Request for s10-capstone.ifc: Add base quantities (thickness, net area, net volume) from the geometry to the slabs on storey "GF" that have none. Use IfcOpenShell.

First a look at what the model holds.

```python
import ifcopenshell
import ifcopenshell.util.element
import ifcopenshell.util.unit

model = ifcopenshell.open("s10-capstone.ifc")
print(model.schema)
for unit_type in ("LENGTHUNIT", "AREAUNIT", "VOLUMEUNIT"):
    print(unit_type, ifcopenshell.util.unit.calculate_unit_scale(model, unit_type))
storey = next(s for s in model.by_type("IfcBuildingStorey") if s.Name == "GF")
slabs = [e for e in ifcopenshell.util.element.get_decomposition(storey) if e.is_a("IfcSlab")]
for e in sorted(slabs, key=lambda e: e.id()):
    print(e.id(), e.is_a(), e.Name, list(ifcopenshell.util.element.get_psets(e, qtos_only=True)), sep=" | ")
```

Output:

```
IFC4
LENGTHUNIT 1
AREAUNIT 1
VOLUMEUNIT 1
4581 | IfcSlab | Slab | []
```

```python
import ifcopenshell
import ifcopenshell.api.pset
import ifcopenshell.geom
import ifcopenshell.util.element
import ifcopenshell.util.shape
import ifcopenshell.util.unit

model = ifcopenshell.open("s10-capstone.ifc")
unit_scale = ifcopenshell.util.unit.calculate_unit_scale(model)
area_scale = ifcopenshell.util.unit.calculate_unit_scale(model, "AREAUNIT")
volume_scale = ifcopenshell.util.unit.calculate_unit_scale(model, "VOLUMEUNIT")
settings = ifcopenshell.geom.settings()

storey = next(s for s in model.by_type("IfcBuildingStorey") if s.Name == "GF")
slabs = [e for e in ifcopenshell.util.element.get_decomposition(storey) if e.is_a("IfcSlab")]

for e in sorted(slabs, key=lambda e: e.id()):
    if ifcopenshell.util.element.get_psets(e, qtos_only=True, should_inherit=False):
        continue
    # Geometry comes back in metres, in the element's own axes.
    shape = ifcopenshell.geom.create_shape(settings, e)
    values = {
        "Width": ifcopenshell.util.shape.get_z(shape.geometry) / unit_scale,
        "NetArea": ifcopenshell.util.shape.get_footprint_area(shape.geometry) / area_scale,
        "NetVolume": ifcopenshell.util.shape.get_volume(shape.geometry) / volume_scale,
    }
    qto = ifcopenshell.api.pset.add_qto(model, product=e, name="Qto_SlabBaseQuantities")
    ifcopenshell.api.pset.edit_qto(model, qto=qto, properties=values)
    print(e.id(), {k: round(v, 3) for k, v in values.items()})

model.write("s10-capstone_edited.ifc")
```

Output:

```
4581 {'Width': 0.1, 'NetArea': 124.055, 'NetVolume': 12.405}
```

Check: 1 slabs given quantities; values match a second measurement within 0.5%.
